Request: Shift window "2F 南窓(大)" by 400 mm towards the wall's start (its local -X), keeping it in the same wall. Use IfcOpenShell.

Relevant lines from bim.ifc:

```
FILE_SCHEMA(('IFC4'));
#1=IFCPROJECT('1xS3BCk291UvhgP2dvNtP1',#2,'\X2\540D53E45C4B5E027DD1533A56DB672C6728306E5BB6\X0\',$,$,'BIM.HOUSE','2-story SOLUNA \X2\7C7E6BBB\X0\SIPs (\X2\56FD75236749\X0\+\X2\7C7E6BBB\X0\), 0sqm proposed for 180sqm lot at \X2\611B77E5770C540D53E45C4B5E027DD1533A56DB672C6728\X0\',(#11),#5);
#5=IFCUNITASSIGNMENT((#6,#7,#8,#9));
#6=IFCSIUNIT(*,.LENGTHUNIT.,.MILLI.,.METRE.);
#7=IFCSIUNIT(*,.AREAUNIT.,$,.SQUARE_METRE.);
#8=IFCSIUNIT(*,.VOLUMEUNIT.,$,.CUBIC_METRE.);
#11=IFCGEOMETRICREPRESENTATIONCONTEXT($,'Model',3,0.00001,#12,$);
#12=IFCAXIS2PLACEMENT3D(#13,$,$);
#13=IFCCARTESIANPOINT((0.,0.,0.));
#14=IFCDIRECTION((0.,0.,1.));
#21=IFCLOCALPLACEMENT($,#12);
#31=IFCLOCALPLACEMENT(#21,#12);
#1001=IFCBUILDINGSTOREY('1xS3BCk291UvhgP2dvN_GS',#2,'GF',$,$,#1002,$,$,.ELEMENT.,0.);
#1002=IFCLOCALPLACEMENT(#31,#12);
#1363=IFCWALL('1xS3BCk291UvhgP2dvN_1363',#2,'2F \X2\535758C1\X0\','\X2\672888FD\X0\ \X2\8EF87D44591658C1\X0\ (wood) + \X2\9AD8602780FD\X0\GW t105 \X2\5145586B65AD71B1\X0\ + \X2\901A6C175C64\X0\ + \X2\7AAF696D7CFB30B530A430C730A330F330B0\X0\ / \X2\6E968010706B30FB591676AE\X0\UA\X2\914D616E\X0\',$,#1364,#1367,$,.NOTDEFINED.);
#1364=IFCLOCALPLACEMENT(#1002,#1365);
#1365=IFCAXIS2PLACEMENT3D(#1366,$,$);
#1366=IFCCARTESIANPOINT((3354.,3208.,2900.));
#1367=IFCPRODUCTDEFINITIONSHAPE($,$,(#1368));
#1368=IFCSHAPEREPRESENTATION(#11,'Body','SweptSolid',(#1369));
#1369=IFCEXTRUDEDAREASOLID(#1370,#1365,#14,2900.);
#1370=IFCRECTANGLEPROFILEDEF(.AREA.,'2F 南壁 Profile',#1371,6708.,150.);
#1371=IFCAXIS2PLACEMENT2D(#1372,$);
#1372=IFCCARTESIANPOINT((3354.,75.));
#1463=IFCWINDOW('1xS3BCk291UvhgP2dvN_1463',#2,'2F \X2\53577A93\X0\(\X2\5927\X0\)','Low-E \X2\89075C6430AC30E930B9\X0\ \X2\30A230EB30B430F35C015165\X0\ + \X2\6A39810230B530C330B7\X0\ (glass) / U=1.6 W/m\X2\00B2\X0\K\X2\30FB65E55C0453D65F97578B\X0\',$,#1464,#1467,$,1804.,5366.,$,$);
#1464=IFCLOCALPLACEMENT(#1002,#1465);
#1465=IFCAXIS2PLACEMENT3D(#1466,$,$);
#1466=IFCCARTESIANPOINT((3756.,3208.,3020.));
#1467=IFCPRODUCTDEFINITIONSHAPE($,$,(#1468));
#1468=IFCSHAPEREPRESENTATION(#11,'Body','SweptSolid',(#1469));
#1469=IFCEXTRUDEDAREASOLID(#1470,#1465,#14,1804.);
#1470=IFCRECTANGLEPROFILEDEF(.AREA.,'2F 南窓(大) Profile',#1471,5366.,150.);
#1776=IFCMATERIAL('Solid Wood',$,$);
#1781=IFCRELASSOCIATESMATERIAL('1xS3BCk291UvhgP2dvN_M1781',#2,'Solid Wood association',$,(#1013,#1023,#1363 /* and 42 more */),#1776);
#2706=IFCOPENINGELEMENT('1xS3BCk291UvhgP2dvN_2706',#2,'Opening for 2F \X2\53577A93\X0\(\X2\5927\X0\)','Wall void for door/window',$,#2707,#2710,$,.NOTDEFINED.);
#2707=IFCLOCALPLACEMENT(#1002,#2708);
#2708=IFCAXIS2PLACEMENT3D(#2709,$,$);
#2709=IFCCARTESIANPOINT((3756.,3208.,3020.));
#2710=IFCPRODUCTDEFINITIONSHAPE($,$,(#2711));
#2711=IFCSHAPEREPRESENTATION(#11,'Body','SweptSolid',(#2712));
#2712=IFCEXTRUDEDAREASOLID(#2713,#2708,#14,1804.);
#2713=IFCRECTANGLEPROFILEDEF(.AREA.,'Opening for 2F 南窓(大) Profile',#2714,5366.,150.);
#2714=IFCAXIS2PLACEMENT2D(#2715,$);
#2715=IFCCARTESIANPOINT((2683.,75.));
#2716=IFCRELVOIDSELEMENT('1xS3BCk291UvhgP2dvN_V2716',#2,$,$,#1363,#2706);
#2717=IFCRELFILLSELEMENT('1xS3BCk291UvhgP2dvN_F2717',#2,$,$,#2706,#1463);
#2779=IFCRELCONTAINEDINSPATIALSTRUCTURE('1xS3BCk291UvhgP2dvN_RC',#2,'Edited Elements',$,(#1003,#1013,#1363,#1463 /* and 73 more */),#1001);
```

```python
import ifcopenshell
import ifcopenshell.api.geometry
import ifcopenshell.util.placement

model = ifcopenshell.open("bim.ifc")

window = model.by_guid("1xS3BCk291UvhgP2dvN_1463")
opening = window.FillsVoids[0].RelatingOpeningElement
wall = opening.VoidsElements[0].RelatingBuildingElement

wall_matrix = ifcopenshell.util.placement.get_local_placement(wall.ObjectPlacement)
shift = wall_matrix[:3, 0] * -400.0
before = ifcopenshell.util.placement.get_local_placement(window.ObjectPlacement)[:3, 3].copy()

# The window is not placed relative to its opening, so move both.
for product in (opening, window):
    matrix = ifcopenshell.util.placement.get_local_placement(product.ObjectPlacement)
    matrix[:3, 3] += shift
    ifcopenshell.api.geometry.edit_object_placement(model, product=product, matrix=matrix, is_si=False)

after = ifcopenshell.util.placement.get_local_placement(window.ObjectPlacement)[:3, 3]
print("window moved by", (after - before).round(3) + 0.0)

model.write("bim_rev.ifc")
```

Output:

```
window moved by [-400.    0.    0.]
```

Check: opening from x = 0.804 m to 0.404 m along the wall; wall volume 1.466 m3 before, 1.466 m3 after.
